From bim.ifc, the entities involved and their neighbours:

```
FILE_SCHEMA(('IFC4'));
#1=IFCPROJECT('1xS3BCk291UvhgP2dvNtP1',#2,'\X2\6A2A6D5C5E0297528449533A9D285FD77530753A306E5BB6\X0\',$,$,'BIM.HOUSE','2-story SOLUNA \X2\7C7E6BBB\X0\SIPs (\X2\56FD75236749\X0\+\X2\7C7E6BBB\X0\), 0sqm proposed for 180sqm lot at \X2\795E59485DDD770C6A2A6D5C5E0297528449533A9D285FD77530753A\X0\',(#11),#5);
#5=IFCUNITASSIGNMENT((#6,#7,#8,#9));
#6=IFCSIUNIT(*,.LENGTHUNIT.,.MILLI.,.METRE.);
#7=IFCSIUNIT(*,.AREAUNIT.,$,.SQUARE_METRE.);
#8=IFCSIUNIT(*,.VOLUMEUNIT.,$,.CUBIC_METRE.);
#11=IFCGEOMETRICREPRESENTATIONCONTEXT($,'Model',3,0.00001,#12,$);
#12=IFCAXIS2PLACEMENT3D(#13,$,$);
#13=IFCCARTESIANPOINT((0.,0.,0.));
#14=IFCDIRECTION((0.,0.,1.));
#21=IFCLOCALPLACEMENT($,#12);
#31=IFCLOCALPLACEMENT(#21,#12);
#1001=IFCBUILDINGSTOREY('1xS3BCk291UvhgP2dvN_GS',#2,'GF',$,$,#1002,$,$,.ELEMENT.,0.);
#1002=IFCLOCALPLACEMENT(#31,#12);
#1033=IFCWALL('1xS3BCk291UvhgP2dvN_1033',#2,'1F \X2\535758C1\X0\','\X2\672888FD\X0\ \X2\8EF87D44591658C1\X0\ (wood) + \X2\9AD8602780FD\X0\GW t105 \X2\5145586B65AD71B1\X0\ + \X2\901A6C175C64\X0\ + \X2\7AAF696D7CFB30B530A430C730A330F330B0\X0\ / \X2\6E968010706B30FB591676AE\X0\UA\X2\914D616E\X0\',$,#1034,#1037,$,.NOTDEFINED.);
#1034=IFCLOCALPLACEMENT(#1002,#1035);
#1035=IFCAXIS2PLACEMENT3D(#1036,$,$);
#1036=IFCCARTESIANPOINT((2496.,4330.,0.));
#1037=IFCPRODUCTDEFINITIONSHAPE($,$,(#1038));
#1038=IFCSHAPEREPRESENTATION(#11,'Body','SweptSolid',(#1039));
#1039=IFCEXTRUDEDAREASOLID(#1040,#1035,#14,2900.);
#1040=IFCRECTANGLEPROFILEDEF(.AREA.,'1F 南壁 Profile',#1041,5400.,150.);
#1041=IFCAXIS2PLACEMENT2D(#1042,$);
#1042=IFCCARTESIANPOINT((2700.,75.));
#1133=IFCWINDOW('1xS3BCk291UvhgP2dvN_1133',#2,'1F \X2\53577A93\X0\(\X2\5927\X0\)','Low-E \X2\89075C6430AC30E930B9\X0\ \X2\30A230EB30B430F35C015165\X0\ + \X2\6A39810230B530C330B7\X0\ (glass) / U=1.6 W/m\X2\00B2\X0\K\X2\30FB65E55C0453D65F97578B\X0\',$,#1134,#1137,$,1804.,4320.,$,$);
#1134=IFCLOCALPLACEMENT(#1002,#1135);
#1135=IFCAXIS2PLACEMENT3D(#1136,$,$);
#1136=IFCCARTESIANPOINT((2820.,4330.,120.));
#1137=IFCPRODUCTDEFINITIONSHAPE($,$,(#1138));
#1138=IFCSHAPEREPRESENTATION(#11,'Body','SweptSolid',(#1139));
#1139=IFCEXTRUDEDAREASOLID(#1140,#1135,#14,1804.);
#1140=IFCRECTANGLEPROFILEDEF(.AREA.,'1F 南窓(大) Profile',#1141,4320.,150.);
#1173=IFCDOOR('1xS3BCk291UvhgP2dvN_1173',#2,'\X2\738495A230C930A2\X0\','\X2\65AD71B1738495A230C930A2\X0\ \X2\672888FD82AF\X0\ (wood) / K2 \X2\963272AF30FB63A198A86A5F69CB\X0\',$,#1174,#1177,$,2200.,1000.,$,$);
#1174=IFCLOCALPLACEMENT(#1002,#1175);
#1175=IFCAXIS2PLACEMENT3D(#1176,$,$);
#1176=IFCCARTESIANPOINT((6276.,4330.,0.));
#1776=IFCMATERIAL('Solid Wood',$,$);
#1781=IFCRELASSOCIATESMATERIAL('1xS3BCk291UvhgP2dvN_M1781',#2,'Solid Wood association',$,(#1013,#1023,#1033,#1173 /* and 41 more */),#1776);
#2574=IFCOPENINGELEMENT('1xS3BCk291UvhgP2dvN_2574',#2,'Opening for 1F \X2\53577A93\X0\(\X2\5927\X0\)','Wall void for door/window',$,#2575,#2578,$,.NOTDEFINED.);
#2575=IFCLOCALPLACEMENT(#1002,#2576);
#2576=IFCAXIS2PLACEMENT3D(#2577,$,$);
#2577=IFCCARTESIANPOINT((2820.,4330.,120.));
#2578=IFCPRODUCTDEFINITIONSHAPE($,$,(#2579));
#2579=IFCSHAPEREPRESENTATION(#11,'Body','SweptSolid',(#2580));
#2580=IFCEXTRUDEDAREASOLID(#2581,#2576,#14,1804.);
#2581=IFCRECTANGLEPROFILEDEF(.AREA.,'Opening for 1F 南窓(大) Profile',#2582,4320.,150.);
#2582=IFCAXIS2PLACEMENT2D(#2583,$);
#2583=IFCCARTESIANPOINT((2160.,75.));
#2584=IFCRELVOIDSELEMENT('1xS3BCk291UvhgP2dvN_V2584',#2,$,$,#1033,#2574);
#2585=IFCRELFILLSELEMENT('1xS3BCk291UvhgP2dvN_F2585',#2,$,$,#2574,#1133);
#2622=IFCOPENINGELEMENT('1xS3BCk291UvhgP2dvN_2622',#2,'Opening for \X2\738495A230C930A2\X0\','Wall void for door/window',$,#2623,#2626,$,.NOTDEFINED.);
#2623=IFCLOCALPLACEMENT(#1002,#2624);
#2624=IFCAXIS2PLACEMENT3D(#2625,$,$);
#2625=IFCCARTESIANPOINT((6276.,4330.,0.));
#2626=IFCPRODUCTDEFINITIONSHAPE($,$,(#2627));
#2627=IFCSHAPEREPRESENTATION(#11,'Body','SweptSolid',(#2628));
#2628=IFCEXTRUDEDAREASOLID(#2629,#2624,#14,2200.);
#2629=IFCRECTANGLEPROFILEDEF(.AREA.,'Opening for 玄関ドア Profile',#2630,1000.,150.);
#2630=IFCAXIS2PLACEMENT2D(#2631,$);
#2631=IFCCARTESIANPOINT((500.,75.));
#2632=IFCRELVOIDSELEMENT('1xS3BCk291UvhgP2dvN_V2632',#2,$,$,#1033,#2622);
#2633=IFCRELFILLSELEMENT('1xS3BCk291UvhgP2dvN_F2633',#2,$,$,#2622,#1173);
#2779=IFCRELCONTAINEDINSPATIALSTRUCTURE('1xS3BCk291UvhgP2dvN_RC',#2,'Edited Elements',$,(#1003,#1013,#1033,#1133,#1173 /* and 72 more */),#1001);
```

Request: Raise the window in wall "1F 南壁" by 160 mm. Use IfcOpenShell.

```python
import numpy as np
import ifcopenshell
import ifcopenshell.api.geometry
import ifcopenshell.util.placement
import ifcopenshell.util.unit

model = ifcopenshell.open("bim.ifc")
unit_scale = ifcopenshell.util.unit.calculate_unit_scale(model)

window = model.by_guid("1xS3BCk291UvhgP2dvN_1133")
opening = window.FillsVoids[0].RelatingOpeningElement
dz = 0.16 / unit_scale

shift = np.array([0.0, 0.0, dz])
# The window is not placed relative to its opening, so move both.
for product in (opening, window):
    matrix = ifcopenshell.util.placement.get_local_placement(product.ObjectPlacement)
    matrix[:3, 3] += shift
    ifcopenshell.api.geometry.edit_object_placement(model, product=product, matrix=matrix, is_si=False)

print(f"moved by {dz * unit_scale:+.3f} m")

model.write("bim_v2.ifc")
```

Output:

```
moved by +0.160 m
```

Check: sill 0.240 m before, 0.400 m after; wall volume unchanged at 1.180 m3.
